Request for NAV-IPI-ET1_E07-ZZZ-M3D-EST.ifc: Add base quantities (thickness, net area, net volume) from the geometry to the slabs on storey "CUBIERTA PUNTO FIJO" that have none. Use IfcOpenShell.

First a look at what the model holds.

```python
import ifcopenshell
import ifcopenshell.util.element
import ifcopenshell.util.unit

model = ifcopenshell.open("NAV-IPI-ET1_E07-ZZZ-M3D-EST.ifc")
print(model.schema)
for unit_type in ("LENGTHUNIT", "AREAUNIT", "VOLUMEUNIT"):
    print(unit_type, ifcopenshell.util.unit.calculate_unit_scale(model, unit_type))
storey = next(s for s in model.by_type("IfcBuildingStorey") if s.Name == "CUBIERTA PUNTO FIJO")
slabs = [e for e in ifcopenshell.util.element.get_decomposition(storey) if e.is_a("IfcSlab")]
for e in sorted(slabs, key=lambda e: e.id()):
    print(e.id(), e.is_a(), e.Name, list(ifcopenshell.util.element.get_psets(e, qtos_only=True)), sep=" | ")
```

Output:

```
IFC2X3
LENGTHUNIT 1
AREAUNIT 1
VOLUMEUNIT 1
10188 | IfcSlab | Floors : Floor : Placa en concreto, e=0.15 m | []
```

```python
import ifcopenshell
import ifcopenshell.api.pset
import ifcopenshell.geom
import ifcopenshell.util.element
import ifcopenshell.util.shape
import ifcopenshell.util.unit

model = ifcopenshell.open("NAV-IPI-ET1_E07-ZZZ-M3D-EST.ifc")
unit_scale = ifcopenshell.util.unit.calculate_unit_scale(model)
area_scale = ifcopenshell.util.unit.calculate_unit_scale(model, "AREAUNIT")
volume_scale = ifcopenshell.util.unit.calculate_unit_scale(model, "VOLUMEUNIT")
settings = ifcopenshell.geom.settings()

storey = next(s for s in model.by_type("IfcBuildingStorey") if s.Name == "CUBIERTA PUNTO FIJO")
slabs = [e for e in ifcopenshell.util.element.get_decomposition(storey) if e.is_a("IfcSlab")]

for e in sorted(slabs, key=lambda e: e.id()):
    if ifcopenshell.util.element.get_psets(e, qtos_only=True, should_inherit=False):
        continue
    # Geometry comes back in metres, in the element's own axes.
    shape = ifcopenshell.geom.create_shape(settings, e)
    values = {
        "Width": ifcopenshell.util.shape.get_z(shape.geometry) / unit_scale,
        "NetArea": ifcopenshell.util.shape.get_footprint_area(shape.geometry) / area_scale,
        "NetVolume": ifcopenshell.util.shape.get_volume(shape.geometry) / volume_scale,
    }
    qto = ifcopenshell.api.pset.add_qto(model, product=e, name="BaseQuantities")
    ifcopenshell.api.pset.edit_qto(model, qto=qto, properties=values)
    print(e.id(), {k: round(v, 3) for k, v in values.items()})

model.write("NAV-IPI-ET1_E07-ZZZ-M3D-EST_updated.ifc")
```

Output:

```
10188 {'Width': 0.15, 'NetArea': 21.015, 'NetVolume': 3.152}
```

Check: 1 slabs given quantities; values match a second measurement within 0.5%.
